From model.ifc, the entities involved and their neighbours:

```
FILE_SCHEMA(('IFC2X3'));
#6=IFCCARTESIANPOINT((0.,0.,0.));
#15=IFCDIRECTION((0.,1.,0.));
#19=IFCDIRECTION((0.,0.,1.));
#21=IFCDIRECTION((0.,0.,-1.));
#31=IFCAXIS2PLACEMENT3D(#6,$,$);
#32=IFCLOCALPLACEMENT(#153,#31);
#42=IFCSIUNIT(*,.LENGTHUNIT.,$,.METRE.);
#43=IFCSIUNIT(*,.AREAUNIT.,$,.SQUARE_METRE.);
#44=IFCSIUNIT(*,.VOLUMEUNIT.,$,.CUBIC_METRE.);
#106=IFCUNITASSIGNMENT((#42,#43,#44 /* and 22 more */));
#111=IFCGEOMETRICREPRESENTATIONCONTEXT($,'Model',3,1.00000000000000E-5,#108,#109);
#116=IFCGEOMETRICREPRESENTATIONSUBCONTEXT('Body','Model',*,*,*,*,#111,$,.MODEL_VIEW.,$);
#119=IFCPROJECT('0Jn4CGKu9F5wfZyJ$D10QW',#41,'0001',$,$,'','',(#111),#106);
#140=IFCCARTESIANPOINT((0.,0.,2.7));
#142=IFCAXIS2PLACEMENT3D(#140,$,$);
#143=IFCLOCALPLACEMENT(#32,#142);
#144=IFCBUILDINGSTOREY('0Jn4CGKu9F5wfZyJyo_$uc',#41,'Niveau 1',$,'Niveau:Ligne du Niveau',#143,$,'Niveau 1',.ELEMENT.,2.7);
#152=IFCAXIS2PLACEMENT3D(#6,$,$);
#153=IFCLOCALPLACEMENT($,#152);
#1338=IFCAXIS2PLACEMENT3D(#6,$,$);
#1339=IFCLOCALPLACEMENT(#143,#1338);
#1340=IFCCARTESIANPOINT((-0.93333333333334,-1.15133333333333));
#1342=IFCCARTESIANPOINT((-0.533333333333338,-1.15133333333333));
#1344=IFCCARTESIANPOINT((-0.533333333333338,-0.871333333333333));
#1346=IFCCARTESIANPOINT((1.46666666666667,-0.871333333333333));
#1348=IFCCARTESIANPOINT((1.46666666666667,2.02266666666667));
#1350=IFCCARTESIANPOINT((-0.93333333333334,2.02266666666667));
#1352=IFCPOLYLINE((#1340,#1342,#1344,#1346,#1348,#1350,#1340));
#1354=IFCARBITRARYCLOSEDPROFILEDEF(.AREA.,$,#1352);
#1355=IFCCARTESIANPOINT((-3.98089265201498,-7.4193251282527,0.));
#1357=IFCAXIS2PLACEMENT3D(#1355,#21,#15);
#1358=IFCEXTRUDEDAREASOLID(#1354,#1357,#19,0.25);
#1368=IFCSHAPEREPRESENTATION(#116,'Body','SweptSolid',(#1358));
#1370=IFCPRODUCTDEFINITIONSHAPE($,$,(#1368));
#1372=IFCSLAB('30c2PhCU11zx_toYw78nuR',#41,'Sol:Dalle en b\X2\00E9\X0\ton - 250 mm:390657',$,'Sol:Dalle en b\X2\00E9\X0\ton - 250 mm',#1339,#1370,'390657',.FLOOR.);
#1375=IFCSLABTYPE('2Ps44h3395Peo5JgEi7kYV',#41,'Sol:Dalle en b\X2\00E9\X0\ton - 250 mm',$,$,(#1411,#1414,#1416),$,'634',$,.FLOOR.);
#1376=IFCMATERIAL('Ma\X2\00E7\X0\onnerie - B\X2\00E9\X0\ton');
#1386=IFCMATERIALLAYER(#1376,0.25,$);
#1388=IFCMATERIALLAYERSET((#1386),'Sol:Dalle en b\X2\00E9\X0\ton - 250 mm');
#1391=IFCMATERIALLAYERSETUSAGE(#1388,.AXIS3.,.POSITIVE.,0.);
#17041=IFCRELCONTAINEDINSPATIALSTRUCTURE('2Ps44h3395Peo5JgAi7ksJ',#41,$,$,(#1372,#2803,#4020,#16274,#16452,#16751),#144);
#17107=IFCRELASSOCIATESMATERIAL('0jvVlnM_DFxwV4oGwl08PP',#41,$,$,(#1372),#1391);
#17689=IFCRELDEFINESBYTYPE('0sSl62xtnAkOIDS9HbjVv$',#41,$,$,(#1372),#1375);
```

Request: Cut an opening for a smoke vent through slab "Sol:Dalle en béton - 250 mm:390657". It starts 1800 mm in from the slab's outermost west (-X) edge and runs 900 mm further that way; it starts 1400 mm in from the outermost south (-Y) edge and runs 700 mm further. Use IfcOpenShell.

```python
import numpy as np
import ifcopenshell
import ifcopenshell.api.feature
import ifcopenshell.api.geometry
import ifcopenshell.api.root
import ifcopenshell.geom
import ifcopenshell.util.placement
import ifcopenshell.util.representation
import ifcopenshell.util.shape
import ifcopenshell.util.unit

model = ifcopenshell.open("model.ifc")
unit_scale = ifcopenshell.util.unit.calculate_unit_scale(model)
settings = ifcopenshell.geom.settings()


def volume(element):
    """Net volume in cubic metres, openings subtracted."""
    shape = ifcopenshell.geom.create_shape(settings, element)
    return ifcopenshell.util.shape.get_volume(shape.geometry)


slab = model.by_id(1372)
before = volume(slab)

# Extent in the slab's own axes, in metres. The edges named are its -X and -Y sides.
slab_shape = ifcopenshell.geom.create_shape(settings, slab)
vertices = ifcopenshell.util.shape.get_vertices(slab_shape.geometry)
x_min, y_min, bottom = vertices.min(axis=0)
top = vertices[:, 2].max()

opening = ifcopenshell.api.root.create_entity(model, ifc_class="IfcOpeningElement", name="Smoke vent opening")
context = ifcopenshell.util.representation.get_context(model, "Model", "Body", "MODEL_VIEW")
width, depth = 0.9, 0.7
outline = [(0.0, 0.0), (width, 0.0), (width, depth), (0.0, depth), (0.0, 0.0)]
# Overshoot both faces by 50 mm so the cut is clean.
shape = ifcopenshell.api.geometry.add_slab_representation(
    model, context=context, depth=top - bottom + 0.1, polyline=outline
)
ifcopenshell.api.geometry.assign_representation(model, product=opening, representation=shape)

matrix = ifcopenshell.util.placement.get_local_placement(slab.ObjectPlacement)
matrix[:, 3] = matrix @ np.append(np.array([x_min + 1.8, y_min + 1.4, bottom - 0.05]) / unit_scale, 1.0)
ifcopenshell.api.geometry.edit_object_placement(model, product=opening, matrix=matrix, is_si=False)
ifcopenshell.api.feature.add_feature(model, feature=opening, element=slab)

after = volume(slab)

print(f"slab volume {before:.3f} -> {after:.3f} m3")

model.write("model-out.ifc")
```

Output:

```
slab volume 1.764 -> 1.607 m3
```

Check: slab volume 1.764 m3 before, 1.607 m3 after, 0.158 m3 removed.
